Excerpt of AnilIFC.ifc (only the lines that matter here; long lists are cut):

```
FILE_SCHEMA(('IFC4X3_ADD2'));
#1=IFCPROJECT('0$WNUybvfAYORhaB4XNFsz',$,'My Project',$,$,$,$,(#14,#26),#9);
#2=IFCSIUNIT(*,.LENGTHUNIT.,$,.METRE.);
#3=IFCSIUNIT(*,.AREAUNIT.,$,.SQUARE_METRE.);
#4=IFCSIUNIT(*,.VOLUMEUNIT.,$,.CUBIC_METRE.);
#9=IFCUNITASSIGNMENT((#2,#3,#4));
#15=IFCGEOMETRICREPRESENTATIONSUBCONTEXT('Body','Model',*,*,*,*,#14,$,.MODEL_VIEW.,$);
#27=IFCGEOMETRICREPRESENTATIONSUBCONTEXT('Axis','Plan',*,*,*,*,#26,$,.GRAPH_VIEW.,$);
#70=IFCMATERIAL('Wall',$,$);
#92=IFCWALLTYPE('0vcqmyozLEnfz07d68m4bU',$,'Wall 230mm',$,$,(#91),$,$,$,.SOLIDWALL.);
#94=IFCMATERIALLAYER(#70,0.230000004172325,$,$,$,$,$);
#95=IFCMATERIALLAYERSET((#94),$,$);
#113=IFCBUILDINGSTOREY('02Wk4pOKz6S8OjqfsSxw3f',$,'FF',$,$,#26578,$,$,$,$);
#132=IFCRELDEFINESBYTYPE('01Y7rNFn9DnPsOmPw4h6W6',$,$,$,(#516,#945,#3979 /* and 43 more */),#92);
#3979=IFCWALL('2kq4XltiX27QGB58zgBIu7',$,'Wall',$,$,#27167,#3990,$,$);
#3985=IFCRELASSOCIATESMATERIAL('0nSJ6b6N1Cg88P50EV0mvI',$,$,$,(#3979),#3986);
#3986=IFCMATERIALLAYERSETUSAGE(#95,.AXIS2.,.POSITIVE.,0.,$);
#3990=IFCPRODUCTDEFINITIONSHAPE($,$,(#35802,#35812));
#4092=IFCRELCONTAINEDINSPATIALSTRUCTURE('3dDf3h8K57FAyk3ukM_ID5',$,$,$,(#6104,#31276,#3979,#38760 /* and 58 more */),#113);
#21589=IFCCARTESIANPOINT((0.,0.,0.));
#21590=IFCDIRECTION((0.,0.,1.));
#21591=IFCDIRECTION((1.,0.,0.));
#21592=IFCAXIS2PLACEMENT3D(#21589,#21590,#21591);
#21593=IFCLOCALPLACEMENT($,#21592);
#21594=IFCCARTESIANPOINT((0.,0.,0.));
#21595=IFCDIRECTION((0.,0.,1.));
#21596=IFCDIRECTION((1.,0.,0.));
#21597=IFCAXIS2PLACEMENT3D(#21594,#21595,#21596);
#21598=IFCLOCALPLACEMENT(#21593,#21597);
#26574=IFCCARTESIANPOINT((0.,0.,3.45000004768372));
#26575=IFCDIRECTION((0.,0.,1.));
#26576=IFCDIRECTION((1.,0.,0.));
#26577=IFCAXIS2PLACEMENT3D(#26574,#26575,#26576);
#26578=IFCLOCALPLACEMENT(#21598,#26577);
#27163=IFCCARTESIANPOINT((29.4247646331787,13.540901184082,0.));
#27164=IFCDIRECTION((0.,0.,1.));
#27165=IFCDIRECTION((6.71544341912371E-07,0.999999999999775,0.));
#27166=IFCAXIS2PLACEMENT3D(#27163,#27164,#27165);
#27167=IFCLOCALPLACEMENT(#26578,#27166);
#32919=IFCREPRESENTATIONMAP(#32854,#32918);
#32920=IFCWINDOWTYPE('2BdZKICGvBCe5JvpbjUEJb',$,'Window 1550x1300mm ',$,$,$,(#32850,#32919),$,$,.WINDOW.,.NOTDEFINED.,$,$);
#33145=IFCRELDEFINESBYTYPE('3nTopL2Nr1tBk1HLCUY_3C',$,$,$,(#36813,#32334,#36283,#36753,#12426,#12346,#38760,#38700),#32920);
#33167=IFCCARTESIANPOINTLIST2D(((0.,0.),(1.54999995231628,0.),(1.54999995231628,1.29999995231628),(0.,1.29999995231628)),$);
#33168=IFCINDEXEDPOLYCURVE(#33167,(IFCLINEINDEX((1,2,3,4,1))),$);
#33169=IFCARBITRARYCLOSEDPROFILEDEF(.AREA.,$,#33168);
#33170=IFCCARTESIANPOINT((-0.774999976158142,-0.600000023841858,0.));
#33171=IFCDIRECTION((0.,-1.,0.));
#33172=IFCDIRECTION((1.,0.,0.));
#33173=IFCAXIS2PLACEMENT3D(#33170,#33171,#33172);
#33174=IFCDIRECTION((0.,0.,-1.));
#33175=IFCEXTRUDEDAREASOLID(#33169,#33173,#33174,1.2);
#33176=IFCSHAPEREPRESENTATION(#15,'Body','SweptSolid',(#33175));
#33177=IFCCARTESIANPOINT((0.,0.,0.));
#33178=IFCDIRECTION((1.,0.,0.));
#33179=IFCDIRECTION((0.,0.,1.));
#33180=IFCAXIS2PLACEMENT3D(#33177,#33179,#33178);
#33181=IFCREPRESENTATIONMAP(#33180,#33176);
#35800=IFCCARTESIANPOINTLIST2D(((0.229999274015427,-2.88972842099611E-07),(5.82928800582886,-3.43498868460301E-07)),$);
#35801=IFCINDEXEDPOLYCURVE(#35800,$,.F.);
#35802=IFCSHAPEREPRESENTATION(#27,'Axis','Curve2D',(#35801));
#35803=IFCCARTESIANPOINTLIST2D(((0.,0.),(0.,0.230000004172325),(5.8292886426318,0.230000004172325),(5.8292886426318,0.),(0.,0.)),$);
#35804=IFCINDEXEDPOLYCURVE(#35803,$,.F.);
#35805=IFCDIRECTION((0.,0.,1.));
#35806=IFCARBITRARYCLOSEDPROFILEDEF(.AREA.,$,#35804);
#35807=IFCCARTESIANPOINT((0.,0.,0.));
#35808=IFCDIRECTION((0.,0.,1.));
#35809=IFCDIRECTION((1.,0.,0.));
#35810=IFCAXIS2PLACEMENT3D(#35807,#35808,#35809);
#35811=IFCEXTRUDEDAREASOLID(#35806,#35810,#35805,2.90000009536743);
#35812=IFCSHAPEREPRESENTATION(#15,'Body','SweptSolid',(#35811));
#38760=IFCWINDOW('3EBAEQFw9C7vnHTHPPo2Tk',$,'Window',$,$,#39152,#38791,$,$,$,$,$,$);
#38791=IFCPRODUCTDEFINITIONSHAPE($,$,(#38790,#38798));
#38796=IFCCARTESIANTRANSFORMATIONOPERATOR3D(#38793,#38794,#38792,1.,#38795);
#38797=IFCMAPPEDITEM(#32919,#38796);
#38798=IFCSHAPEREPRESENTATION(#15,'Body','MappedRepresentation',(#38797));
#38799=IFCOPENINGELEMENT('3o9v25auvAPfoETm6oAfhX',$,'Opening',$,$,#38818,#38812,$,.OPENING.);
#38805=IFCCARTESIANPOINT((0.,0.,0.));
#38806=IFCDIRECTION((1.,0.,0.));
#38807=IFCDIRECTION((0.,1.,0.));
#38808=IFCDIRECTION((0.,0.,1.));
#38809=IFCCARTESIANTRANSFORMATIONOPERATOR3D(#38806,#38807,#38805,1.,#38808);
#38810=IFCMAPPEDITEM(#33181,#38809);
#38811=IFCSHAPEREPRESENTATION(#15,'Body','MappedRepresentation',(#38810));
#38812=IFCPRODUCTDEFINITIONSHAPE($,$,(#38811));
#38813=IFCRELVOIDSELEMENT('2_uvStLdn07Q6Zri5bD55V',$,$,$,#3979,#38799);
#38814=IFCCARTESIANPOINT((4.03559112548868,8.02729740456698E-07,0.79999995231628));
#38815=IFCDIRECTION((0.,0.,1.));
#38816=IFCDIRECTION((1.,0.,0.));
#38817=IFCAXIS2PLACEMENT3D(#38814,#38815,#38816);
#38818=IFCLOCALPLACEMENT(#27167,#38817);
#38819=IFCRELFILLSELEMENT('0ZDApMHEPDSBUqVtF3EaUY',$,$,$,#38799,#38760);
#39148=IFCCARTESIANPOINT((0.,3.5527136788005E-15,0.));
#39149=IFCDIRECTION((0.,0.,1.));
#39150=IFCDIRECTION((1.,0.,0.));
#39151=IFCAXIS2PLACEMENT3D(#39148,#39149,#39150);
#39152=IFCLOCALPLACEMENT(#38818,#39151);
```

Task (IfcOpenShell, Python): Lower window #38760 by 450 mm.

```python
import numpy as np
import ifcopenshell
import ifcopenshell.api.geometry
import ifcopenshell.util.placement
import ifcopenshell.util.unit

model = ifcopenshell.open("AnilIFC.ifc")
unit_scale = ifcopenshell.util.unit.calculate_unit_scale(model)

window = model.by_guid("3EBAEQFw9C7vnHTHPPo2Tk")
opening = window.FillsVoids[0].RelatingOpeningElement
dz = -0.45 / unit_scale

shift = np.array([0.0, 0.0, dz])
# The window is placed relative to its opening, so it follows when the opening moves.
matrix = ifcopenshell.util.placement.get_local_placement(opening.ObjectPlacement)
matrix[:3, 3] += shift
ifcopenshell.api.geometry.edit_object_placement(
    model, product=opening, matrix=matrix, is_si=False, should_transform_children=True
)

print(f"moved by {dz * unit_scale:+.3f} m")

model.write("AnilIFC_rev.ifc")
```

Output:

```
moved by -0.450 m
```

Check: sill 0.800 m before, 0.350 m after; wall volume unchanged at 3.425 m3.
